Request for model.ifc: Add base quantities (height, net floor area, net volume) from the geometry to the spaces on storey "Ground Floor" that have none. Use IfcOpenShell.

First a look at what the model holds.

```python
import ifcopenshell
import ifcopenshell.util.element
import ifcopenshell.util.unit

model = ifcopenshell.open("model.ifc")
print(model.schema)
for unit_type in ("LENGTHUNIT", "AREAUNIT", "VOLUMEUNIT"):
    print(unit_type, ifcopenshell.util.unit.calculate_unit_scale(model, unit_type))
storey = next(s for s in model.by_type("IfcBuildingStorey") if s.Name == "Ground Floor")
spaces = [e for e in ifcopenshell.util.element.get_decomposition(storey) if e.is_a("IfcSpace")]
for e in sorted(spaces, key=lambda e: e.id()):
    print(e.id(), e.is_a(), e.Name, list(ifcopenshell.util.element.get_psets(e, qtos_only=True)), sep=" | ")
```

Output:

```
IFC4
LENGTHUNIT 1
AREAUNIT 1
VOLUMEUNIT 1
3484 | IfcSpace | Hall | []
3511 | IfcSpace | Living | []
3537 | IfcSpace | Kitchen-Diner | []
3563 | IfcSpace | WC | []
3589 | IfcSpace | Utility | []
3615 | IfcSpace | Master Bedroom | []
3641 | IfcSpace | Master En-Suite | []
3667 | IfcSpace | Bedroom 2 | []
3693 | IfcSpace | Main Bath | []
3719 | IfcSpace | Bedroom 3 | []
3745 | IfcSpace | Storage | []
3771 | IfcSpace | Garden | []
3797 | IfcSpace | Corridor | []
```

```python
import ifcopenshell
import ifcopenshell.api.pset
import ifcopenshell.geom
import ifcopenshell.util.element
import ifcopenshell.util.shape
import ifcopenshell.util.unit

model = ifcopenshell.open("model.ifc")
unit_scale = ifcopenshell.util.unit.calculate_unit_scale(model)
area_scale = ifcopenshell.util.unit.calculate_unit_scale(model, "AREAUNIT")
volume_scale = ifcopenshell.util.unit.calculate_unit_scale(model, "VOLUMEUNIT")
settings = ifcopenshell.geom.settings()

storey = next(s for s in model.by_type("IfcBuildingStorey") if s.Name == "Ground Floor")
spaces = [e for e in ifcopenshell.util.element.get_decomposition(storey) if e.is_a("IfcSpace")]

for e in sorted(spaces, key=lambda e: e.id()):
    if ifcopenshell.util.element.get_psets(e, qtos_only=True, should_inherit=False):
        continue
    # Geometry comes back in metres, in the element's own axes.
    shape = ifcopenshell.geom.create_shape(settings, e)
    values = {
        "Height": ifcopenshell.util.shape.get_z(shape.geometry) / unit_scale,
        "NetFloorArea": ifcopenshell.util.shape.get_footprint_area(shape.geometry) / area_scale,
        "NetVolume": ifcopenshell.util.shape.get_volume(shape.geometry) / volume_scale,
    }
    qto = ifcopenshell.api.pset.add_qto(model, product=e, name="Qto_SpaceBaseQuantities")
    ifcopenshell.api.pset.edit_qto(model, qto=qto, properties=values)
    print(e.id(), {k: round(v, 3) for k, v in values.items()})

model.write("model-out.ifc")
```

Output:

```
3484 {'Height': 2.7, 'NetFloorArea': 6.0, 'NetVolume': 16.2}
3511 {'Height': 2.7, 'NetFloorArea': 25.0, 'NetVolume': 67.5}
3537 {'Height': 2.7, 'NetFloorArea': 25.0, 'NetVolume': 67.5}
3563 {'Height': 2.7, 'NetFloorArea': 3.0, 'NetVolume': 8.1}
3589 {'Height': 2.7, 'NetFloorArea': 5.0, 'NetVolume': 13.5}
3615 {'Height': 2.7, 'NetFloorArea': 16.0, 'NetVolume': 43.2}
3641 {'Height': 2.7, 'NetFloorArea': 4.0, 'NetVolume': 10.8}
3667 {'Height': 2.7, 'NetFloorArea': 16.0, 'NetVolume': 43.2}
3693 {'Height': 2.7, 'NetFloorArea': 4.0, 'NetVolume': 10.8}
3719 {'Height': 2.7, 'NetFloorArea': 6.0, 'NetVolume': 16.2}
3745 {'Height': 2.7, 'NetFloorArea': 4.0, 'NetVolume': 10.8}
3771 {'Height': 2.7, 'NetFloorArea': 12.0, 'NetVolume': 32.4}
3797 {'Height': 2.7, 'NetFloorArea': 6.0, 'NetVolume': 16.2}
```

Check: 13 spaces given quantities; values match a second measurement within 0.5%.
